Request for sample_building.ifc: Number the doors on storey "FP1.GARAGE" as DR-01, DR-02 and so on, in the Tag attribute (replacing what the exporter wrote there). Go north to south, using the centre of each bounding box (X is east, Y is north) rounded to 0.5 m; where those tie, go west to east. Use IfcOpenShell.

First a look at what the model holds.

```python
import ifcopenshell
import ifcopenshell.util.element
import ifcopenshell.util.placement

model = ifcopenshell.open("sample_building.ifc")
print(model.schema)
storey = next(s for s in model.by_type("IfcBuildingStorey") if s.Name == "FP1.GARAGE")
doors = [e for e in ifcopenshell.util.element.get_decomposition(storey) if e.is_a("IfcDoor")]
for e in sorted(doors, key=lambda e: e.id()):
    origin = ifcopenshell.util.placement.get_local_placement(e.ObjectPlacement)[:3, 3]
    print(e.id(), e.Tag, e.Name, origin.round(2) + 0.0, sep=" | ")
```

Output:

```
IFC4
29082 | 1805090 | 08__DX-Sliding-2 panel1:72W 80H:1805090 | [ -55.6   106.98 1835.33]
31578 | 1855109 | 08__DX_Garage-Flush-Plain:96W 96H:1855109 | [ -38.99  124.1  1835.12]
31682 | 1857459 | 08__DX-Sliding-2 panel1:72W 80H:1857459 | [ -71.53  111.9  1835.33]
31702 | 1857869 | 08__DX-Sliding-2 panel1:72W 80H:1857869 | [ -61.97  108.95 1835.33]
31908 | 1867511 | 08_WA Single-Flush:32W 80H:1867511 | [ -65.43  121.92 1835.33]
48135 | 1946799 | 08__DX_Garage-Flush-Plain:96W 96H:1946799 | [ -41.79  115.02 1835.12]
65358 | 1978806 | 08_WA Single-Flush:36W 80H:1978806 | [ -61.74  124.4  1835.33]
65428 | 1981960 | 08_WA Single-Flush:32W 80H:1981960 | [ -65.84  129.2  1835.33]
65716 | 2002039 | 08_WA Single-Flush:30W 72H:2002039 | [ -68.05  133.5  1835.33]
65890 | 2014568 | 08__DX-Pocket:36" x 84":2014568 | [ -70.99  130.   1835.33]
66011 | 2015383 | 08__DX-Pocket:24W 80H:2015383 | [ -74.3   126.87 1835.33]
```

```python
import ifcopenshell
import ifcopenshell.geom
import ifcopenshell.util.element
import ifcopenshell.util.shape

model = ifcopenshell.open("sample_building.ifc")
settings = ifcopenshell.geom.settings()
settings.set("use-world-coords", True)


def centre(element):
    shape = ifcopenshell.geom.create_shape(settings, element)
    return ifcopenshell.util.shape.get_bbox_centroid(shape.geometry)


storey = next(s for s in model.by_type("IfcBuildingStorey") if s.Name == "FP1.GARAGE")
doors = [e for e in ifcopenshell.util.element.get_decomposition(storey) if e.is_a("IfcDoor")]

# Insertion points can sit at a corner or the storey origin, so sort by the geometry (in metres).
centres = {e: centre(e) for e in doors}
doors.sort(key=lambda e: (-round(centres[e][1] / 0.5), centres[e][0]))

for i, e in enumerate(doors, start=1):
    number = f"DR-{i:02d}"
    e.Tag = number
    print(e.id(), number)

model.write("sample_building_v2.ifc")
```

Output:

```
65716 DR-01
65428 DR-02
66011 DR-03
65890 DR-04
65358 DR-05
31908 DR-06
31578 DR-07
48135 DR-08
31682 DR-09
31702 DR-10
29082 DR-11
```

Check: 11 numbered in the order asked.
